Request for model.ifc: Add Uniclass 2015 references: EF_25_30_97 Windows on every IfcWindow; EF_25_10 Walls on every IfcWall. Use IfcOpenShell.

First a look at what the model holds.

```python
import ifcopenshell

model = ifcopenshell.open("model.ifc")
print(model.schema)
print("classifications:", [c.Name for c in model.by_type("IfcClassification")])
for ifc_class in ("IfcDoor", "IfcRoof", "IfcStair", "IfcWall", "IfcWindow"):
    print(ifc_class, len(model.by_type(ifc_class)))
```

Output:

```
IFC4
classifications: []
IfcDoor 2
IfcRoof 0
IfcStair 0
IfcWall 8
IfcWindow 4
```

```python
import ifcopenshell
import ifcopenshell.api.classification

model = ifcopenshell.open("model.ifc")

system = ifcopenshell.api.classification.add_classification(model, classification="Uniclass 2015")

codes = {
    "IfcWindow": ("EF_25_30_97", "Windows"),
    "IfcWall": ("EF_25_10", "Walls"),
}
for ifc_class, (code, name) in codes.items():
    products = model.by_type(ifc_class)
    ifcopenshell.api.classification.add_reference(
        model, products=products, classification=system, identification=code, name=name
    )
    print(code, len(products))

model.write("model_rev.ifc")
```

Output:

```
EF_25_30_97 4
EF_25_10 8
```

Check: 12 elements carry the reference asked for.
